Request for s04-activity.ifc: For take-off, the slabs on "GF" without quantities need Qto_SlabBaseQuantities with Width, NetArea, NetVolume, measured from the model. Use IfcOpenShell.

First a look at what the model holds.

```python
import ifcopenshell
import ifcopenshell.util.element
import ifcopenshell.util.unit

model = ifcopenshell.open("s04-activity.ifc")
print(model.schema)
for unit_type in ("LENGTHUNIT", "AREAUNIT", "VOLUMEUNIT"):
    print(unit_type, ifcopenshell.util.unit.calculate_unit_scale(model, unit_type))
storey = next(s for s in model.by_type("IfcBuildingStorey") if s.Name == "GF")
slabs = [e for e in ifcopenshell.util.element.get_decomposition(storey) if e.is_a("IfcSlab")]
for e in sorted(slabs, key=lambda e: e.id()):
    print(e.id(), e.is_a(), e.Name, list(ifcopenshell.util.element.get_psets(e, qtos_only=True)), sep=" | ")
```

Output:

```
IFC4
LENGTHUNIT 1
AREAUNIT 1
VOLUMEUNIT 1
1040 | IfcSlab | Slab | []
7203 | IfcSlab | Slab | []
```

```python
import ifcopenshell
import ifcopenshell.api.pset
import ifcopenshell.geom
import ifcopenshell.util.element
import ifcopenshell.util.shape
import ifcopenshell.util.unit

model = ifcopenshell.open("s04-activity.ifc")
unit_scale = ifcopenshell.util.unit.calculate_unit_scale(model)
area_scale = ifcopenshell.util.unit.calculate_unit_scale(model, "AREAUNIT")
volume_scale = ifcopenshell.util.unit.calculate_unit_scale(model, "VOLUMEUNIT")
settings = ifcopenshell.geom.settings()

storey = next(s for s in model.by_type("IfcBuildingStorey") if s.Name == "GF")
slabs = [e for e in ifcopenshell.util.element.get_decomposition(storey) if e.is_a("IfcSlab")]

for e in sorted(slabs, key=lambda e: e.id()):
    if ifcopenshell.util.element.get_psets(e, qtos_only=True, should_inherit=False):
        continue
    # Geometry comes back in metres, in the element's own axes.
    shape = ifcopenshell.geom.create_shape(settings, e)
    values = {
        "Width": ifcopenshell.util.shape.get_z(shape.geometry) / unit_scale,
        "NetArea": ifcopenshell.util.shape.get_footprint_area(shape.geometry) / area_scale,
        "NetVolume": ifcopenshell.util.shape.get_volume(shape.geometry) / volume_scale,
    }
    qto = ifcopenshell.api.pset.add_qto(model, product=e, name="Qto_SlabBaseQuantities")
    ifcopenshell.api.pset.edit_qto(model, qto=qto, properties=values)
    print(e.id(), {k: round(v, 3) for k, v in values.items()})

model.write("s04-activity_v2.ifc")
```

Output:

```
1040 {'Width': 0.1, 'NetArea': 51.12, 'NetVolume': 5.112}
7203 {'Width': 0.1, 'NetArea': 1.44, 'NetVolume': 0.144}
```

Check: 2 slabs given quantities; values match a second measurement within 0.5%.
